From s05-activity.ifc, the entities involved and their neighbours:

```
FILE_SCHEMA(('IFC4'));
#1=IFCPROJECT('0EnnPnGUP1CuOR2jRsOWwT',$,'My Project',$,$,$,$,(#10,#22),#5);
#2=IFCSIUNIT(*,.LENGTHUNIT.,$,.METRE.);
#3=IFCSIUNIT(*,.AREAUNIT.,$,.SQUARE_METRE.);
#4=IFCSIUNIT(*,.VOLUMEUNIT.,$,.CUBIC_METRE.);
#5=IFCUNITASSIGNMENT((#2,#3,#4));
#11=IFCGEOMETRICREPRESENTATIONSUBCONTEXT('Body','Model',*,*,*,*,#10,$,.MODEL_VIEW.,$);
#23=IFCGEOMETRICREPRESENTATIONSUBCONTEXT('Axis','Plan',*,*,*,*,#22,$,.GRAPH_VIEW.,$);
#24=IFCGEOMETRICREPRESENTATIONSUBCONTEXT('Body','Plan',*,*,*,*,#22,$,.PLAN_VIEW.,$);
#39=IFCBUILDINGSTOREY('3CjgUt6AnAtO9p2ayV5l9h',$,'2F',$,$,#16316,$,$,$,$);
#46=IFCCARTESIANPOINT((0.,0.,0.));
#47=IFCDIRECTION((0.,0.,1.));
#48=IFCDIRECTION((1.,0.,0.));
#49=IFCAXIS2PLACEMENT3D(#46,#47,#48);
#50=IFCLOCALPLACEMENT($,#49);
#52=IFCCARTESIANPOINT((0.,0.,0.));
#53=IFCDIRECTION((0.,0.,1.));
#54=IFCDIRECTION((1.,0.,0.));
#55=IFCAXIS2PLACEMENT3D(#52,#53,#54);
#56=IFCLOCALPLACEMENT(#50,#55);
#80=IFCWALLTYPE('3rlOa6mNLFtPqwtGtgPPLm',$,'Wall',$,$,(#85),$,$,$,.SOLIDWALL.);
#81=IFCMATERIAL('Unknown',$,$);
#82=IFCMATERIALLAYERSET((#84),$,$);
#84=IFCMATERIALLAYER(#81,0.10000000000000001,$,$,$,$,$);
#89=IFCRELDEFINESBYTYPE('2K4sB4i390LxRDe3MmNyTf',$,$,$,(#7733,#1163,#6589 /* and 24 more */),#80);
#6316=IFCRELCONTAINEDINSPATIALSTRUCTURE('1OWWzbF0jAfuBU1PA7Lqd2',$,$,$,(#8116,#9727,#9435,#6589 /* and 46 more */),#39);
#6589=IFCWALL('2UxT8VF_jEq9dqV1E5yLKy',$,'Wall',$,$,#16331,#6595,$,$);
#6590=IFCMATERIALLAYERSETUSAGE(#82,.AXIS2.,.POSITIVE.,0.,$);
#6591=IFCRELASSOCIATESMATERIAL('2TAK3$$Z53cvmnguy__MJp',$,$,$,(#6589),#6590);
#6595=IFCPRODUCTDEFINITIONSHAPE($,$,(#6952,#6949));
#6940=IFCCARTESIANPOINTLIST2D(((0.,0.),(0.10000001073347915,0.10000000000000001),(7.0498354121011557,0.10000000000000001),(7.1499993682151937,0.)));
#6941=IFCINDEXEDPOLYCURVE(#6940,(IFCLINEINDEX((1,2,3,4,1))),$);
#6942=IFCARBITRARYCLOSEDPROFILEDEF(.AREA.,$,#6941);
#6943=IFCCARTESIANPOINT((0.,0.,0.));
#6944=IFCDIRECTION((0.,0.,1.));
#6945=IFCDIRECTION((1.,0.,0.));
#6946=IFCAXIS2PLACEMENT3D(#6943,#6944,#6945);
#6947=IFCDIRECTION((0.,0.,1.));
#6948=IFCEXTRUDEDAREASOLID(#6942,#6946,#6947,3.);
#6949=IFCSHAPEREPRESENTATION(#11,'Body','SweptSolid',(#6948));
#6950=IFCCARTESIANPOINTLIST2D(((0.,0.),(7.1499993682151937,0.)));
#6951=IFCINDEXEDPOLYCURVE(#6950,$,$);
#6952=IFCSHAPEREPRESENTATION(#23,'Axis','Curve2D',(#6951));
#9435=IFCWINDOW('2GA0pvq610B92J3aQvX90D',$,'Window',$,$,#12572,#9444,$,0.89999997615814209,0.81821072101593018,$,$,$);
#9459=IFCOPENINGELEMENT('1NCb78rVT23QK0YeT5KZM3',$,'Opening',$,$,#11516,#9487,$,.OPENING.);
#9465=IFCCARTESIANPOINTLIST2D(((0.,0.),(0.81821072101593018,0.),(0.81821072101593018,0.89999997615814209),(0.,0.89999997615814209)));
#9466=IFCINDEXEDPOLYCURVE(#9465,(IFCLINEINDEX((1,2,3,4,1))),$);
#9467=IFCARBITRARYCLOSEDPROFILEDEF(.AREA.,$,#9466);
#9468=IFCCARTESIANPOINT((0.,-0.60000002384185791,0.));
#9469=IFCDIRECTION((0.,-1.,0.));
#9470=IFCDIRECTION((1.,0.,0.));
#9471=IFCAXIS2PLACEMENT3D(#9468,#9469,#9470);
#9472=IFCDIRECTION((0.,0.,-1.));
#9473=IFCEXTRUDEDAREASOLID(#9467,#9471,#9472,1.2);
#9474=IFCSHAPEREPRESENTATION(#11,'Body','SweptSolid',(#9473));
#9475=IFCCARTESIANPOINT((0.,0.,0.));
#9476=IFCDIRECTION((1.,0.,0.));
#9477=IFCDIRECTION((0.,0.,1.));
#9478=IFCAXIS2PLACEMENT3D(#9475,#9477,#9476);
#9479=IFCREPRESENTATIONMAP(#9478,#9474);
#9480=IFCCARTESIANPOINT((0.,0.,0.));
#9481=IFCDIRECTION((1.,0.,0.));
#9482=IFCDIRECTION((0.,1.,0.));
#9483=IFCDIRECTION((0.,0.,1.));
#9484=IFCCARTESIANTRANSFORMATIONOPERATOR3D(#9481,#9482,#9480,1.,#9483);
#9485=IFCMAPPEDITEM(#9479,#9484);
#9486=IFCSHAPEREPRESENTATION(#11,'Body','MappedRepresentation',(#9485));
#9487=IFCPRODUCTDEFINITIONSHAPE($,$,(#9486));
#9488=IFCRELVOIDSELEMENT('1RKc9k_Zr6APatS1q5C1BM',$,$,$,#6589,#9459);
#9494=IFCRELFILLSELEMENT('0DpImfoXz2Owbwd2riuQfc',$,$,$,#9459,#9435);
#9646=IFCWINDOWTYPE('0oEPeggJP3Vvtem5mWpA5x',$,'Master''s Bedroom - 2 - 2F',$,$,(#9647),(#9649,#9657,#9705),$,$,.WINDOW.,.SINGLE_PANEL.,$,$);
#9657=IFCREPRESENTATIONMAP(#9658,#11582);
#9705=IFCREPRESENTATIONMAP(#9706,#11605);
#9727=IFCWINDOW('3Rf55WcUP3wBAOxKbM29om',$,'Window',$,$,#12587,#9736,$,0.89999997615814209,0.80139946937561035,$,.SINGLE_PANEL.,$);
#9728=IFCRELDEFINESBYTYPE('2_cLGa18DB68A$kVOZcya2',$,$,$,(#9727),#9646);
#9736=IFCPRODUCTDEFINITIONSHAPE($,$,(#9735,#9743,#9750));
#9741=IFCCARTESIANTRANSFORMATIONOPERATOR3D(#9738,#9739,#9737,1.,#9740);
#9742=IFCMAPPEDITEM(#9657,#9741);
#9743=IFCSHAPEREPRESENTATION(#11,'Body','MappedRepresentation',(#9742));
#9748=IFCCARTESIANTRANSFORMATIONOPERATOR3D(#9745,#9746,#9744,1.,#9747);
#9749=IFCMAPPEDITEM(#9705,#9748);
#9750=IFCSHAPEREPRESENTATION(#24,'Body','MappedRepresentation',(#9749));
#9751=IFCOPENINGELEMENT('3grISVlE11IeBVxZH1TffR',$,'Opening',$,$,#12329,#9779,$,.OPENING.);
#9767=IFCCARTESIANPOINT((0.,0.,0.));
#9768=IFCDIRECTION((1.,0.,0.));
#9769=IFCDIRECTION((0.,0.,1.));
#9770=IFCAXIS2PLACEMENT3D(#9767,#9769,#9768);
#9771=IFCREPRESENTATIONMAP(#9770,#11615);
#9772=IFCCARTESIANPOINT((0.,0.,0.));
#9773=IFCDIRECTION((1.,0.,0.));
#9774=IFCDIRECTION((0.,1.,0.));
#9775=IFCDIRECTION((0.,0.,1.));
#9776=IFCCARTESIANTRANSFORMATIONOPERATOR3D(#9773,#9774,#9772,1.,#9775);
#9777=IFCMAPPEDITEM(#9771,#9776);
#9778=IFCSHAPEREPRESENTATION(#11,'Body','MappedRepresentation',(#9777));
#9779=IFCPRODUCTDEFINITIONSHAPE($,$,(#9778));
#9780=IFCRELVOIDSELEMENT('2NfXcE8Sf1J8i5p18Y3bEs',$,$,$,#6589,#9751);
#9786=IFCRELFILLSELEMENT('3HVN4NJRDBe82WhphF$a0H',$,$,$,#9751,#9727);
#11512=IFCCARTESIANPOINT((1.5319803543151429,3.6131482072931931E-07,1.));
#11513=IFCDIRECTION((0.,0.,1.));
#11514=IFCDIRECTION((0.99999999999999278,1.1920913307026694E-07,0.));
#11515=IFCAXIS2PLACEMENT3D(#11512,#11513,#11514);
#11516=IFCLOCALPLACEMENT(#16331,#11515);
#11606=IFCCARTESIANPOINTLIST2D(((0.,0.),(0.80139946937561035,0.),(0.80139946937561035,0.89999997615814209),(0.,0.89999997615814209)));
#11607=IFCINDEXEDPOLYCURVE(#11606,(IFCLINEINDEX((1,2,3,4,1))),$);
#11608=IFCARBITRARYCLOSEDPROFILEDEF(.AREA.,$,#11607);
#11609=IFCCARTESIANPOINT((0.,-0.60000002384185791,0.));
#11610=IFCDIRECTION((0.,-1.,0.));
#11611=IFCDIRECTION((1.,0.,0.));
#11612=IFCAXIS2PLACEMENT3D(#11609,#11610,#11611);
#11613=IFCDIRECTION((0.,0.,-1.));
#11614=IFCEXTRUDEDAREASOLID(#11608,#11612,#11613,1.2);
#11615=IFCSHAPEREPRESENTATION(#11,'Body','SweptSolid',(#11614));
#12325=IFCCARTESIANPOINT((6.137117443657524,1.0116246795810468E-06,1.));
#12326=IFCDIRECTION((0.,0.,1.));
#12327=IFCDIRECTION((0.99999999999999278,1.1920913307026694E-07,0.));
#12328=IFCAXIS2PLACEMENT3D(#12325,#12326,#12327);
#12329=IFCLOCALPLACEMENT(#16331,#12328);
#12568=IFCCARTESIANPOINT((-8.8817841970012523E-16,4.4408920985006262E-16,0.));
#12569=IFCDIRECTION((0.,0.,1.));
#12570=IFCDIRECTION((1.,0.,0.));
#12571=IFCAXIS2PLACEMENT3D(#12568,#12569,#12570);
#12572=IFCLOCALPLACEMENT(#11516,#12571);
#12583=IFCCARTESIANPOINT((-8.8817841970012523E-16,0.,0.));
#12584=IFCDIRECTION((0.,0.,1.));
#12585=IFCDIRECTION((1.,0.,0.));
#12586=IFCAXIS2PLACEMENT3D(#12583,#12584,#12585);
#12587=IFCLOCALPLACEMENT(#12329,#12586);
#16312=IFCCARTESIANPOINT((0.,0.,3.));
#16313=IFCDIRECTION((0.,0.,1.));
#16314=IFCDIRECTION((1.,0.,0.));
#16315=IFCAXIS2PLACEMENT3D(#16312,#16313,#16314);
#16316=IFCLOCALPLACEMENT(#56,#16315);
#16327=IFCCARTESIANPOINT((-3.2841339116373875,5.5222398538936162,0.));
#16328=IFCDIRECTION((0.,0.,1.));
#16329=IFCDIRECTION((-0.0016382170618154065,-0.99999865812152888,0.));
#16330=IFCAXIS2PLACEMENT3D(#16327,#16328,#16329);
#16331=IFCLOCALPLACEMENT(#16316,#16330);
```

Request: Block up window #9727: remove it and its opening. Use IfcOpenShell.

```python
import ifcopenshell
import ifcopenshell.api.feature
import ifcopenshell.api.root
import ifcopenshell.geom
import ifcopenshell.util.shape

model = ifcopenshell.open("s05-activity.ifc")
settings = ifcopenshell.geom.settings()


def volume(element):
    """Net volume in cubic metres, openings subtracted."""
    shape = ifcopenshell.geom.create_shape(settings, element)
    return ifcopenshell.util.shape.get_volume(shape.geometry)


window = model.by_guid("3Rf55WcUP3wBAOxKbM29om")
opening = window.FillsVoids[0].RelatingOpeningElement
wall = opening.VoidsElements[0].RelatingBuildingElement
before = volume(wall)

ifcopenshell.api.root.remove_product(model, product=window)
ifcopenshell.api.feature.remove_feature(model, feature=opening)

after = volume(wall)

print(f"wall volume {before:.3f} -> {after:.3f} m3")

model.write("s05-activity_v2.ifc")
```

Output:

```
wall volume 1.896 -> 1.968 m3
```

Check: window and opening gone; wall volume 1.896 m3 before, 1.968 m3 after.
